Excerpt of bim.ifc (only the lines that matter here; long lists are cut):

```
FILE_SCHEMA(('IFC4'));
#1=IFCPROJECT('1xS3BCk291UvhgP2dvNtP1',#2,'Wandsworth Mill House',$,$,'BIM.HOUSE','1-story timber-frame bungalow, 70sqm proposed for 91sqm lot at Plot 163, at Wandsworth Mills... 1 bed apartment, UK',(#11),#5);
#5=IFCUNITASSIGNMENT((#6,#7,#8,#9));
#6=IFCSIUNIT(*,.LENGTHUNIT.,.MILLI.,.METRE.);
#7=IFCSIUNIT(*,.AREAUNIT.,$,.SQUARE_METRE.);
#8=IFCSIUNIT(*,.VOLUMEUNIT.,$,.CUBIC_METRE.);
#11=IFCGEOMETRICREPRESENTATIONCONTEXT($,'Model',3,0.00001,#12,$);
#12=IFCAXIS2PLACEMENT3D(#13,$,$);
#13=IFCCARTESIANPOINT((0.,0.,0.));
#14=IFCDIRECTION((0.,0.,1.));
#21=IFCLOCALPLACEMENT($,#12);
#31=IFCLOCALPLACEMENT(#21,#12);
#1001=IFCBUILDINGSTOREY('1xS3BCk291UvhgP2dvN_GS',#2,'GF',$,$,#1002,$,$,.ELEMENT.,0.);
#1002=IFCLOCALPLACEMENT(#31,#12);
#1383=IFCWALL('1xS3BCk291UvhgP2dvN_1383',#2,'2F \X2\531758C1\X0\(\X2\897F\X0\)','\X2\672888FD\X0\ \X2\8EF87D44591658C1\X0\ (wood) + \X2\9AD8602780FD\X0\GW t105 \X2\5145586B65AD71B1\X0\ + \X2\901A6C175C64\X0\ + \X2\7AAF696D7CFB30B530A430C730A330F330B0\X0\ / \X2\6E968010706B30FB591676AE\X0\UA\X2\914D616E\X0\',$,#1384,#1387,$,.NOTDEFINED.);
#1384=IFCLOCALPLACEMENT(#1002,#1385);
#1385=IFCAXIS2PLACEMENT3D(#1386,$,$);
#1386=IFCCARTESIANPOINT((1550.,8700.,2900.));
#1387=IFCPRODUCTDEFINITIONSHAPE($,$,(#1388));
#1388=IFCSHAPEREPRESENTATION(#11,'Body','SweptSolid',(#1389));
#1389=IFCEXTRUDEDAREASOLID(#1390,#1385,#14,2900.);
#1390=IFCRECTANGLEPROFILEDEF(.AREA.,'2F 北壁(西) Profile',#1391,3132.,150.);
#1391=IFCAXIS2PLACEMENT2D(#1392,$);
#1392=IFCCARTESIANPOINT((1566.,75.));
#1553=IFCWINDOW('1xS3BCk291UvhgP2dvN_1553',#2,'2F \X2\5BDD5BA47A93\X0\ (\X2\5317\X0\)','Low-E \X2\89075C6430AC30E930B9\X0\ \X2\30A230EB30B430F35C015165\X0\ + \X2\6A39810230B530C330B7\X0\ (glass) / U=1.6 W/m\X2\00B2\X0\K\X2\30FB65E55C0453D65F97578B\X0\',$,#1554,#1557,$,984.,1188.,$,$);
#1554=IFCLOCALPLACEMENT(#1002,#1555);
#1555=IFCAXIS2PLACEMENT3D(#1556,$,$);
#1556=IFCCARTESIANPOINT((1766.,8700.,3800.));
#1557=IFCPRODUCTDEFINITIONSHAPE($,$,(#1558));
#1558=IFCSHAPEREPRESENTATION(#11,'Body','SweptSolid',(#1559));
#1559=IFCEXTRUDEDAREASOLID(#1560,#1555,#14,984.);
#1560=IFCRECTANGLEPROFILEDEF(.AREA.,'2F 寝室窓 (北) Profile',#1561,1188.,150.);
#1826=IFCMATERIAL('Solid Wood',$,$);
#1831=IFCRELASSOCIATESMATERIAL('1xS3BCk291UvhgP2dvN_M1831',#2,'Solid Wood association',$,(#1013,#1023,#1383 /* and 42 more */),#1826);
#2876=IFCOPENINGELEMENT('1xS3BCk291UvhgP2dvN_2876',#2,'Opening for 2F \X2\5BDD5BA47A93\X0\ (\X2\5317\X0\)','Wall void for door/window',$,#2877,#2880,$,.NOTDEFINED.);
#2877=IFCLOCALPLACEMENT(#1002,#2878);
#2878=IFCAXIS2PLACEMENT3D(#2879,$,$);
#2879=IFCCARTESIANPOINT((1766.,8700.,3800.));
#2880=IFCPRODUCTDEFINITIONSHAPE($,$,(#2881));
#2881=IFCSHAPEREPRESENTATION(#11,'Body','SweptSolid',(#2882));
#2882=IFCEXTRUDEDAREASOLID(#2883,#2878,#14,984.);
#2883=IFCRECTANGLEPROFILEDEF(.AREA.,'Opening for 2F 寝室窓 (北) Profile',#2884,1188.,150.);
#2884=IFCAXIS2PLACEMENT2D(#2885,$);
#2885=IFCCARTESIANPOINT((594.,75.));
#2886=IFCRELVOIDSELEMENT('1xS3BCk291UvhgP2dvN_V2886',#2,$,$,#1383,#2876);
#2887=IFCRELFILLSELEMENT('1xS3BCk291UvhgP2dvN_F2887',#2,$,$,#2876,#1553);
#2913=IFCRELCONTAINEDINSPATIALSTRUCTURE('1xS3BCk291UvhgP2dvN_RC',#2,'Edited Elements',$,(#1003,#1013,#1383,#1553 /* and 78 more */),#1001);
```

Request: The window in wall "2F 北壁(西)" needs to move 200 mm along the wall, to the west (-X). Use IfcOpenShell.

```python
import ifcopenshell
import ifcopenshell.api.geometry
import ifcopenshell.util.placement

model = ifcopenshell.open("bim.ifc")

window = model.by_guid("1xS3BCk291UvhgP2dvN_1553")
opening = window.FillsVoids[0].RelatingOpeningElement
wall = opening.VoidsElements[0].RelatingBuildingElement

wall_matrix = ifcopenshell.util.placement.get_local_placement(wall.ObjectPlacement)
shift = wall_matrix[:3, 0] * -200.0
before = ifcopenshell.util.placement.get_local_placement(window.ObjectPlacement)[:3, 3].copy()

# The window is not placed relative to its opening, so move both.
for product in (opening, window):
    matrix = ifcopenshell.util.placement.get_local_placement(product.ObjectPlacement)
    matrix[:3, 3] += shift
    ifcopenshell.api.geometry.edit_object_placement(model, product=product, matrix=matrix, is_si=False)

after = ifcopenshell.util.placement.get_local_placement(window.ObjectPlacement)[:3, 3]
print("window moved by", (after - before).round(3) + 0.0)

model.write("bim_updated.ifc")
```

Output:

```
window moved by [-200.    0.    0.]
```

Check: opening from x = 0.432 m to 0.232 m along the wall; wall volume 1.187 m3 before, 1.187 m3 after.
